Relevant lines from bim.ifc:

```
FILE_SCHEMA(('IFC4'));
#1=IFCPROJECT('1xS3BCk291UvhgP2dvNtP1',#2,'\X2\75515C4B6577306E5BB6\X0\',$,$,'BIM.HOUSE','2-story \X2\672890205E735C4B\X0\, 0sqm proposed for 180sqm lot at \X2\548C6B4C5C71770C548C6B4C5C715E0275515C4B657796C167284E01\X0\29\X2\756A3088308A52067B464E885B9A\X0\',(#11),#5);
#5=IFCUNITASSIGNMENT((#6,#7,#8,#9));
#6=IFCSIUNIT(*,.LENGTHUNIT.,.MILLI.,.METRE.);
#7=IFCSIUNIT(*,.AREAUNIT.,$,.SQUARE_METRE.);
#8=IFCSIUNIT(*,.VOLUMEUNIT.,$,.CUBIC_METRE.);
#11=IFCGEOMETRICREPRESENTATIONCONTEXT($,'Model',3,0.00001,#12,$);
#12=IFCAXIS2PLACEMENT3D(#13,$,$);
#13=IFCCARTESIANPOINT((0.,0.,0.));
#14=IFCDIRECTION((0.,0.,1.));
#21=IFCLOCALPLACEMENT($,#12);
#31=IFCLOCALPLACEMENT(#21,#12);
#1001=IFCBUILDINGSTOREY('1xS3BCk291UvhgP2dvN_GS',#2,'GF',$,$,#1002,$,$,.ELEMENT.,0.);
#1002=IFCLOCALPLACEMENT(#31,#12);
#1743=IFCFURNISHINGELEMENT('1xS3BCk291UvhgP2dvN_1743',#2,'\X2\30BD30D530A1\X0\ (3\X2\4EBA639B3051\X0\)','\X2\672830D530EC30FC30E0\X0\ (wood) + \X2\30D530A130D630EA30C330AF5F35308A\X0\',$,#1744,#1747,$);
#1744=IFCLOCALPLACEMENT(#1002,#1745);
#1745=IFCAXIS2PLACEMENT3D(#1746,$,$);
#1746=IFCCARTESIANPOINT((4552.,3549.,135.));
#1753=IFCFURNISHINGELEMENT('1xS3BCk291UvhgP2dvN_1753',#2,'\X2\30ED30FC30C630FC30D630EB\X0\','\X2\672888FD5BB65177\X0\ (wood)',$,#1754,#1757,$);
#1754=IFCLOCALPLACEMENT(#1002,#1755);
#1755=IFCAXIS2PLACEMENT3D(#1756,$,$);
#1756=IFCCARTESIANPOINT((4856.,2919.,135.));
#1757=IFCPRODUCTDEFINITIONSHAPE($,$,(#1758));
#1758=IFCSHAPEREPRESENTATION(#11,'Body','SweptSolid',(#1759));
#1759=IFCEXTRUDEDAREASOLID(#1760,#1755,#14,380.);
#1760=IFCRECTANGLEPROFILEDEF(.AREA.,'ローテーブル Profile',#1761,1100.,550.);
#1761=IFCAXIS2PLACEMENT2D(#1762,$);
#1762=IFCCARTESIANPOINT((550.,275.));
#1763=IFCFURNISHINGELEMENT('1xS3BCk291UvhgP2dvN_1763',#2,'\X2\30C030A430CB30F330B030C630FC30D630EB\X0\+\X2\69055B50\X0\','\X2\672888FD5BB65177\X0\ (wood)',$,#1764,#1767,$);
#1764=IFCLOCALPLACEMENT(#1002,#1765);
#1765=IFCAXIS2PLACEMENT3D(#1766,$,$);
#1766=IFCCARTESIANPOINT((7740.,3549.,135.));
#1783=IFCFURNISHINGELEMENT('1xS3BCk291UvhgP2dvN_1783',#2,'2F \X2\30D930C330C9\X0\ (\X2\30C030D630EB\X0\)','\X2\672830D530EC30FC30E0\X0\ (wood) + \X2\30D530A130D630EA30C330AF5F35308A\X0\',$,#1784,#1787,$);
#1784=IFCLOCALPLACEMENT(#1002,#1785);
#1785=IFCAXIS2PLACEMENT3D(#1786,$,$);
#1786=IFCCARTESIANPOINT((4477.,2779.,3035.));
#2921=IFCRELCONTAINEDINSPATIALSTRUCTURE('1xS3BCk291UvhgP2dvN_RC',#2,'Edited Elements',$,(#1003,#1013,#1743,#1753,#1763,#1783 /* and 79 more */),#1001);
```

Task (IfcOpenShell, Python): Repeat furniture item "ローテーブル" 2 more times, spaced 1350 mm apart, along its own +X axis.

```python
import ifcopenshell
import ifcopenshell.api.geometry
import ifcopenshell.api.root
import ifcopenshell.util.element
import ifcopenshell.util.placement
import ifcopenshell.util.unit

model = ifcopenshell.open("bim.ifc")
unit_scale = ifcopenshell.util.unit.calculate_unit_scale(model)


def reuse_history(source, copy):
    """copy_class also copies each property set's owner history, people and application; keep the originals."""
    for rel in copy.IsDefinedBy:
        if rel.is_a("IfcRelDefinesByProperties") and (history := rel.RelatingPropertyDefinition.OwnerHistory):
            rel.RelatingPropertyDefinition.OwnerHistory = source.OwnerHistory
            ifcopenshell.util.element.remove_deep2(model, history)


source = model.by_guid("1xS3BCk291UvhgP2dvN_1753")
base = ifcopenshell.util.placement.get_local_placement(source.ObjectPlacement)
step = base[:3, 0] * 1.35 / unit_scale

for i in range(1, 3):
    copy = ifcopenshell.api.root.copy_class(model, product=source)
    copy.Representation = ifcopenshell.util.element.copy_deep(
        model, source.Representation, exclude=["IfcGeometricRepresentationContext", "IfcRepresentationMap"]
    )
    reuse_history(source, copy)
    matrix = base.copy()
    matrix[:3, 3] += i * step
    print("added at", matrix[:3, 3].round(3) + 0.0)
    ifcopenshell.api.geometry.edit_object_placement(model, product=copy, matrix=matrix, is_si=False)

model.write("bim_rev.ifc")
```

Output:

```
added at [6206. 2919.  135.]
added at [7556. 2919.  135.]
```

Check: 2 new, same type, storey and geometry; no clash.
